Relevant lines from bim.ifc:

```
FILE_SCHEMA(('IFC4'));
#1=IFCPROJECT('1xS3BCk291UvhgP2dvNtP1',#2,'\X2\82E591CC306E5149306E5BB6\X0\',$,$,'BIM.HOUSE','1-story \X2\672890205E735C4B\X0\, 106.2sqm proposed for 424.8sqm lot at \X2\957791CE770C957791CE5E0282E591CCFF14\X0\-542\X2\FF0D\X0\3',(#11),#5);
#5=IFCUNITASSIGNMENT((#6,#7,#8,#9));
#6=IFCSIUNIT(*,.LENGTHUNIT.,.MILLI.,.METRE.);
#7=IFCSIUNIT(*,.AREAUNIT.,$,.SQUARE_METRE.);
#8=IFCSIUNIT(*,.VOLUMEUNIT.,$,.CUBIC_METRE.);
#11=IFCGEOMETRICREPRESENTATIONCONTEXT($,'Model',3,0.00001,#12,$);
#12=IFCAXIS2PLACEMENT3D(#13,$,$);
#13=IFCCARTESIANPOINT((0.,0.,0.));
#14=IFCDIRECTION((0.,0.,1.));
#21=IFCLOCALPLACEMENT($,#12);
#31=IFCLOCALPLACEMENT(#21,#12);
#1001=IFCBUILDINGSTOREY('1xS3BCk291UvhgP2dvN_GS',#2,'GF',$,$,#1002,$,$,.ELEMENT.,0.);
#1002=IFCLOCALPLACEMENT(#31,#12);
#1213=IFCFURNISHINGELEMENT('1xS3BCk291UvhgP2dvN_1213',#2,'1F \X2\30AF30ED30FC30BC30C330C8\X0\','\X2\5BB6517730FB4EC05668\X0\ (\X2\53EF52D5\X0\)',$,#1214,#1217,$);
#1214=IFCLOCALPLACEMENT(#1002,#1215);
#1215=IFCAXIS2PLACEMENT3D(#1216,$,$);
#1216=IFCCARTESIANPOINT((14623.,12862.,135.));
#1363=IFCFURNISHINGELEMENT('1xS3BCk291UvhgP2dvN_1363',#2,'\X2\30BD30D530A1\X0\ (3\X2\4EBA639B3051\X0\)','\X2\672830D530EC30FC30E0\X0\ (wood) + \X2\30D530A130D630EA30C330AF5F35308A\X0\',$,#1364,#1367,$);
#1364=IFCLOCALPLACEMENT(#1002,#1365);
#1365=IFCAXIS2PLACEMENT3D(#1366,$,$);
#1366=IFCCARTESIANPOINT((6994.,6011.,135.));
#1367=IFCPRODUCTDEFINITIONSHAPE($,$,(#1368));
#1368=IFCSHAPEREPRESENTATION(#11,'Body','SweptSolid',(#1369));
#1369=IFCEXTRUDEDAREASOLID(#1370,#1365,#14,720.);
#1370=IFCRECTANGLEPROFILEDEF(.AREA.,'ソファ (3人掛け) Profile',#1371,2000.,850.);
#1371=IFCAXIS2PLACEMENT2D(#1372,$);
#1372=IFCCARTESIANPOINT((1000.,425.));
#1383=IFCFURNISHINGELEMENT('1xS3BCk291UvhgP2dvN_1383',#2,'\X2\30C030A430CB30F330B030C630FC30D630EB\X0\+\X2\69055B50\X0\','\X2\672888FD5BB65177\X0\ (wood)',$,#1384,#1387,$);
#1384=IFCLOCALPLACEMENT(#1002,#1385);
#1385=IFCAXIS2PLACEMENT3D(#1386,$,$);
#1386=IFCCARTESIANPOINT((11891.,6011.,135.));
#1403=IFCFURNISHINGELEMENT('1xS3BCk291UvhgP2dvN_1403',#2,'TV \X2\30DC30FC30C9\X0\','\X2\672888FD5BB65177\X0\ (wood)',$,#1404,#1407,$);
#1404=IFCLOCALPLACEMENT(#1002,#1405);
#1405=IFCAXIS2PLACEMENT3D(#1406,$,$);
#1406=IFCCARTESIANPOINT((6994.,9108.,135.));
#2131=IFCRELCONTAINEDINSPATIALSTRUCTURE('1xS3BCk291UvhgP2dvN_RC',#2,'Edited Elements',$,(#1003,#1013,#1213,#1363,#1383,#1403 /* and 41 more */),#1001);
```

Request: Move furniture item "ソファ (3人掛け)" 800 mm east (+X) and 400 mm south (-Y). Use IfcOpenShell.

```python
import ifcopenshell
import ifcopenshell.api.geometry
import ifcopenshell.util.placement

model = ifcopenshell.open("bim.ifc")

item = model.by_guid("1xS3BCk291UvhgP2dvN_1363")
matrix = ifcopenshell.util.placement.get_local_placement(item.ObjectPlacement)
matrix[0, 3] += 800.0
matrix[1, 3] -= 400.0
ifcopenshell.api.geometry.edit_object_placement(model, product=item, matrix=matrix, is_si=False)

print(ifcopenshell.util.placement.get_local_placement(item.ObjectPlacement).round(3) + 0.0)

model.write("bim-out.ifc")
```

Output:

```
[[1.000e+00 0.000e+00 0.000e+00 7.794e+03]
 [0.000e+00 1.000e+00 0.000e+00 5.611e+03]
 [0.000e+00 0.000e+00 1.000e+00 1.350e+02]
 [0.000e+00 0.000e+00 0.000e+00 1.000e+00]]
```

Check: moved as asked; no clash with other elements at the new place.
